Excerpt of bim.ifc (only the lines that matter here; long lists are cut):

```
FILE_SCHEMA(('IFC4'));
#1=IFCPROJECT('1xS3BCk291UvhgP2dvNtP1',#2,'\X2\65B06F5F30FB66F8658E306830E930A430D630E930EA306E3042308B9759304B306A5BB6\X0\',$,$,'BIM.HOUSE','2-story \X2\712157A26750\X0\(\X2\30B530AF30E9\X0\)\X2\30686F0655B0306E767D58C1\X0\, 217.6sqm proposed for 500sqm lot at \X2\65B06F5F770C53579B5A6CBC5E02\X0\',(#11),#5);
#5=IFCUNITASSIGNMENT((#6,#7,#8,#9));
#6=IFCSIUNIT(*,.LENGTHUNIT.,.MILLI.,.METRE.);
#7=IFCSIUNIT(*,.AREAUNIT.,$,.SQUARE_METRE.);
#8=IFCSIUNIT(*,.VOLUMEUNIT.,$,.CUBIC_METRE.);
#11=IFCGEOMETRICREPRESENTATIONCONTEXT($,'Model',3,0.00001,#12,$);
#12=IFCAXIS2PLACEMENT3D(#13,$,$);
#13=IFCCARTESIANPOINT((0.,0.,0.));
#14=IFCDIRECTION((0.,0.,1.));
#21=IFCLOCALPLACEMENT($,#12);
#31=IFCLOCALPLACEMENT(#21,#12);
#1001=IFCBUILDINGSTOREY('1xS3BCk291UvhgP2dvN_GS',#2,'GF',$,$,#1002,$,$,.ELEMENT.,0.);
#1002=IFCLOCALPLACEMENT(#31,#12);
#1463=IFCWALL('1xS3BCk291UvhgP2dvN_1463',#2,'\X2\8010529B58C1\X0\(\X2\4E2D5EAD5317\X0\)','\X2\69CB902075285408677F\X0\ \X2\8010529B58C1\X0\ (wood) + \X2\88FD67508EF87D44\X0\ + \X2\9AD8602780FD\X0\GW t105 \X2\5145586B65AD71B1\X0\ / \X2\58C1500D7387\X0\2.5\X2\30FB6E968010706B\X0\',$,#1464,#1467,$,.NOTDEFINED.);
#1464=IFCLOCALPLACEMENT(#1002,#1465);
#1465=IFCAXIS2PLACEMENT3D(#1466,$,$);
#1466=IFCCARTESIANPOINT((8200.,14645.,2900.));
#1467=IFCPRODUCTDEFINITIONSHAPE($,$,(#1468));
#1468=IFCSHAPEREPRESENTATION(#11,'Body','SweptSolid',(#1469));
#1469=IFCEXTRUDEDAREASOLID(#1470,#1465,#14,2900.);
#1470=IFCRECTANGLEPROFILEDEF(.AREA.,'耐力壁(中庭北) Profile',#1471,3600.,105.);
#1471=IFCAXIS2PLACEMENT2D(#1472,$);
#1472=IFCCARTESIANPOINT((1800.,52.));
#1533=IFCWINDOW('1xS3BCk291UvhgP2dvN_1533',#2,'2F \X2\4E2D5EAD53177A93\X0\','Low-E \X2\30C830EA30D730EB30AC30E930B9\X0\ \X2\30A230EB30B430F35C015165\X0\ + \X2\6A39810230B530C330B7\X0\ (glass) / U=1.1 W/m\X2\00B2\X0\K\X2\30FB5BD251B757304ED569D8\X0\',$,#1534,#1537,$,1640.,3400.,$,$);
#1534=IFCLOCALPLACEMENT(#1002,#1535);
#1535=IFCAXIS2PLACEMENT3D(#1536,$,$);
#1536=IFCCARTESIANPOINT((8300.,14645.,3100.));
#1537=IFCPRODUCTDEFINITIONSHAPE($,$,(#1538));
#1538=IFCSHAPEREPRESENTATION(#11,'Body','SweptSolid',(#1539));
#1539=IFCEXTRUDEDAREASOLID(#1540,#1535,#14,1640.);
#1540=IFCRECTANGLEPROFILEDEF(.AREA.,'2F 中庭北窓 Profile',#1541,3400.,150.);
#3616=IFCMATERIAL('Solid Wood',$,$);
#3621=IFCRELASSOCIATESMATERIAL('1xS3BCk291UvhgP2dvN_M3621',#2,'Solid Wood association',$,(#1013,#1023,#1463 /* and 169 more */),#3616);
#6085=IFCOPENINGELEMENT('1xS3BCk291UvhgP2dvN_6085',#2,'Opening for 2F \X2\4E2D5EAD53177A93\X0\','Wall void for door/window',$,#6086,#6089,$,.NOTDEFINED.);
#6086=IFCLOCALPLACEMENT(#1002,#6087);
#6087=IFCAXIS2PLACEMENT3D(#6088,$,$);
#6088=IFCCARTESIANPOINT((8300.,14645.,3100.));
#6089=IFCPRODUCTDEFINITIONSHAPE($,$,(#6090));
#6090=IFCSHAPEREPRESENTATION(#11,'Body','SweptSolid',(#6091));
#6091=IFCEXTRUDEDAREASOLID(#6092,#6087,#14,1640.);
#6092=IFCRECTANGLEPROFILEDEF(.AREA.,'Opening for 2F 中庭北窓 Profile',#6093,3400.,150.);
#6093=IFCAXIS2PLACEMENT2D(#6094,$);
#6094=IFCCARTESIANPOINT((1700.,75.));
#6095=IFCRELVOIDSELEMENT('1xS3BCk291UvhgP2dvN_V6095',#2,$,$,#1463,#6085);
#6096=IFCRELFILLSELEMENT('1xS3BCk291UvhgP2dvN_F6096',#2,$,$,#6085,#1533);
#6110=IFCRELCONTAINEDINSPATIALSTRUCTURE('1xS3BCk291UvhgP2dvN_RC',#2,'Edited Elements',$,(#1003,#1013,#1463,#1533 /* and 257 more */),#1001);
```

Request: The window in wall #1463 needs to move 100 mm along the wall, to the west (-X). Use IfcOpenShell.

```python
import ifcopenshell
import ifcopenshell.api.geometry
import ifcopenshell.util.placement
import ifcopenshell.util.unit

model = ifcopenshell.open("bim.ifc")
unit_scale = ifcopenshell.util.unit.calculate_unit_scale(model)

window = model.by_id(1533)
opening = window.FillsVoids[0].RelatingOpeningElement
wall = opening.VoidsElements[0].RelatingBuildingElement

wall_matrix = ifcopenshell.util.placement.get_local_placement(wall.ObjectPlacement)
shift = wall_matrix[:3, 0] * -0.1 / unit_scale
before = ifcopenshell.util.placement.get_local_placement(window.ObjectPlacement)[:3, 3].copy()

# The window is not placed relative to its opening, so move both.
for product in (opening, window):
    matrix = ifcopenshell.util.placement.get_local_placement(product.ObjectPlacement)
    matrix[:3, 3] += shift
    ifcopenshell.api.geometry.edit_object_placement(model, product=product, matrix=matrix, is_si=False)

after = ifcopenshell.util.placement.get_local_placement(window.ObjectPlacement)[:3, 3]
print("window moved by", (after - before).round(3) + 0.0)

model.write("bim_edited.ifc")
```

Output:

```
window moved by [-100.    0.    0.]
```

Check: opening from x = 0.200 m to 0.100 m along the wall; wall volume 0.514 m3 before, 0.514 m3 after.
